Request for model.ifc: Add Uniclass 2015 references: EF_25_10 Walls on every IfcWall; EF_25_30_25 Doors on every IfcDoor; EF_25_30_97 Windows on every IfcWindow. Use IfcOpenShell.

First a look at what the model holds.

```python
import ifcopenshell

model = ifcopenshell.open("model.ifc")
print(model.schema)
print("classifications:", [c.Name for c in model.by_type("IfcClassification")])
for ifc_class in ("IfcDoor", "IfcRoof", "IfcStair", "IfcWall", "IfcWindow"):
    print(ifc_class, len(model.by_type(ifc_class)))
```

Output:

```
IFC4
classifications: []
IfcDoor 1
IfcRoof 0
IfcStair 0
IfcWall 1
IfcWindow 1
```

```python
import ifcopenshell
import ifcopenshell.api.classification

model = ifcopenshell.open("model.ifc")

system = ifcopenshell.api.classification.add_classification(model, classification="Uniclass 2015")

codes = {
    "IfcWall": ("EF_25_10", "Walls"),
    "IfcDoor": ("EF_25_30_25", "Doors"),
    "IfcWindow": ("EF_25_30_97", "Windows"),
}
for ifc_class, (code, name) in codes.items():
    products = model.by_type(ifc_class)
    ifcopenshell.api.classification.add_reference(
        model, products=products, classification=system, identification=code, name=name
    )
    print(code, len(products))

model.write("model_rev.ifc")
```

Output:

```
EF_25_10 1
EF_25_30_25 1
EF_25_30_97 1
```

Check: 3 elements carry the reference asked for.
